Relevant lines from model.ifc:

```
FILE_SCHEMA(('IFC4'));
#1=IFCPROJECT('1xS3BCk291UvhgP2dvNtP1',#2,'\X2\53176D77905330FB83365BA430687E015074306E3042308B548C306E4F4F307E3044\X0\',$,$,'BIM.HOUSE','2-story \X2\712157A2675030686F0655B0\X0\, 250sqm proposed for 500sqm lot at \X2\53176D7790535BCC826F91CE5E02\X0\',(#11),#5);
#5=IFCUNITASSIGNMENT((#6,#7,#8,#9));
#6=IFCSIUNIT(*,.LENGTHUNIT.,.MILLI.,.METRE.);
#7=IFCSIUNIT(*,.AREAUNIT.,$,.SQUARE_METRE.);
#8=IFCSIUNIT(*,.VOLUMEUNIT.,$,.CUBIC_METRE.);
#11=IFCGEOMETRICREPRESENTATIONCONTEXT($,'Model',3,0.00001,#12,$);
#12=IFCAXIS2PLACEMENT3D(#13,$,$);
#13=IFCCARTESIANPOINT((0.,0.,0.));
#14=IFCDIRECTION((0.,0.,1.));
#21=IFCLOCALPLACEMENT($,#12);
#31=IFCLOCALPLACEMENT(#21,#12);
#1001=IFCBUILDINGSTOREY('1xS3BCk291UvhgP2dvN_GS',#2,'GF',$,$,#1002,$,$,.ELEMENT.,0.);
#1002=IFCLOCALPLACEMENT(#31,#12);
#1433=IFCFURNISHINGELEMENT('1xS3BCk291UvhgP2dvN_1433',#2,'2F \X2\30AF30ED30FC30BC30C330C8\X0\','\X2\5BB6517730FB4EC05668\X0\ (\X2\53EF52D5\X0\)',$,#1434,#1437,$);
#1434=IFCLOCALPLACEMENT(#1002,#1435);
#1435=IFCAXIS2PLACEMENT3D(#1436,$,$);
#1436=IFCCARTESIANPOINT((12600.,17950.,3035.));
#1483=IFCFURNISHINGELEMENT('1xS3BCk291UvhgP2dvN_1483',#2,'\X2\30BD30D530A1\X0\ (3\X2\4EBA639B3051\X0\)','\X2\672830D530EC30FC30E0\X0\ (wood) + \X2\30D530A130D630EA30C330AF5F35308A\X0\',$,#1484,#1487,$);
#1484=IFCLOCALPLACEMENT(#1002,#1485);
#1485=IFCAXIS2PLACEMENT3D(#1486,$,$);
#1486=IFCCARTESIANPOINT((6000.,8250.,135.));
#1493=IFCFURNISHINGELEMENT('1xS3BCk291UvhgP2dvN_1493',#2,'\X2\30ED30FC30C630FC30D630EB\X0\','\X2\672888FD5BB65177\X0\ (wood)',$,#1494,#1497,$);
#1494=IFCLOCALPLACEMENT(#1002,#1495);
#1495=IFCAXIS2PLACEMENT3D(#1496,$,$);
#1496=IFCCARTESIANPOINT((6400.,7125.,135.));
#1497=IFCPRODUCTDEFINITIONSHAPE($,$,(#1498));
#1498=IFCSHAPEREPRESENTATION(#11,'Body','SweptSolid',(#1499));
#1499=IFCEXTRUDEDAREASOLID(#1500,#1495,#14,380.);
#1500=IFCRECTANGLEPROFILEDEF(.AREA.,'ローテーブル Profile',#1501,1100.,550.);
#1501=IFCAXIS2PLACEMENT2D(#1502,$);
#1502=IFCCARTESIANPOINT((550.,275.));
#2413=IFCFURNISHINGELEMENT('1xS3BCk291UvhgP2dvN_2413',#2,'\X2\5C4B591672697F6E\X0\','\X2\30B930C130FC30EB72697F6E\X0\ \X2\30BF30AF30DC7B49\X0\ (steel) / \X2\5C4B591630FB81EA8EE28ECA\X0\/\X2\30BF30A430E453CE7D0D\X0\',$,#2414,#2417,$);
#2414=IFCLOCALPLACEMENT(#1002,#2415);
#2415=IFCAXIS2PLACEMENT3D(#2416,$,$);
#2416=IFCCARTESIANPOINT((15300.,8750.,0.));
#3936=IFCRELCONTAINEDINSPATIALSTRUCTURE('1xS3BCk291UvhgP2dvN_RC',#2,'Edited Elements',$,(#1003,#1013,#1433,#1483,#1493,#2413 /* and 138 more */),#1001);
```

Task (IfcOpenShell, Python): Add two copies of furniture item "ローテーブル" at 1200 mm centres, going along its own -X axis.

```python
import ifcopenshell
import ifcopenshell.api.geometry
import ifcopenshell.api.root
import ifcopenshell.util.element
import ifcopenshell.util.placement
import ifcopenshell.util.unit

model = ifcopenshell.open("model.ifc")
unit_scale = ifcopenshell.util.unit.calculate_unit_scale(model)


def reuse_history(source, copy):
    """copy_class also copies each property set's owner history, people and application; keep the originals."""
    for rel in copy.IsDefinedBy:
        if rel.is_a("IfcRelDefinesByProperties") and (history := rel.RelatingPropertyDefinition.OwnerHistory):
            rel.RelatingPropertyDefinition.OwnerHistory = source.OwnerHistory
            ifcopenshell.util.element.remove_deep2(model, history)


source = model.by_id(1493)
base = ifcopenshell.util.placement.get_local_placement(source.ObjectPlacement)
step = -base[:3, 0] * 1.2 / unit_scale

for i in range(1, 3):
    copy = ifcopenshell.api.root.copy_class(model, product=source)
    copy.Representation = ifcopenshell.util.element.copy_deep(
        model, source.Representation, exclude=["IfcGeometricRepresentationContext", "IfcRepresentationMap"]
    )
    reuse_history(source, copy)
    matrix = base.copy()
    matrix[:3, 3] += i * step
    print("added at", matrix[:3, 3].round(3) + 0.0)
    ifcopenshell.api.geometry.edit_object_placement(model, product=copy, matrix=matrix, is_si=False)

model.write("model_v2.ifc")
```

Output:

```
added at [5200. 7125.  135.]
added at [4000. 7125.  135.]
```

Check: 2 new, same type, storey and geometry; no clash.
